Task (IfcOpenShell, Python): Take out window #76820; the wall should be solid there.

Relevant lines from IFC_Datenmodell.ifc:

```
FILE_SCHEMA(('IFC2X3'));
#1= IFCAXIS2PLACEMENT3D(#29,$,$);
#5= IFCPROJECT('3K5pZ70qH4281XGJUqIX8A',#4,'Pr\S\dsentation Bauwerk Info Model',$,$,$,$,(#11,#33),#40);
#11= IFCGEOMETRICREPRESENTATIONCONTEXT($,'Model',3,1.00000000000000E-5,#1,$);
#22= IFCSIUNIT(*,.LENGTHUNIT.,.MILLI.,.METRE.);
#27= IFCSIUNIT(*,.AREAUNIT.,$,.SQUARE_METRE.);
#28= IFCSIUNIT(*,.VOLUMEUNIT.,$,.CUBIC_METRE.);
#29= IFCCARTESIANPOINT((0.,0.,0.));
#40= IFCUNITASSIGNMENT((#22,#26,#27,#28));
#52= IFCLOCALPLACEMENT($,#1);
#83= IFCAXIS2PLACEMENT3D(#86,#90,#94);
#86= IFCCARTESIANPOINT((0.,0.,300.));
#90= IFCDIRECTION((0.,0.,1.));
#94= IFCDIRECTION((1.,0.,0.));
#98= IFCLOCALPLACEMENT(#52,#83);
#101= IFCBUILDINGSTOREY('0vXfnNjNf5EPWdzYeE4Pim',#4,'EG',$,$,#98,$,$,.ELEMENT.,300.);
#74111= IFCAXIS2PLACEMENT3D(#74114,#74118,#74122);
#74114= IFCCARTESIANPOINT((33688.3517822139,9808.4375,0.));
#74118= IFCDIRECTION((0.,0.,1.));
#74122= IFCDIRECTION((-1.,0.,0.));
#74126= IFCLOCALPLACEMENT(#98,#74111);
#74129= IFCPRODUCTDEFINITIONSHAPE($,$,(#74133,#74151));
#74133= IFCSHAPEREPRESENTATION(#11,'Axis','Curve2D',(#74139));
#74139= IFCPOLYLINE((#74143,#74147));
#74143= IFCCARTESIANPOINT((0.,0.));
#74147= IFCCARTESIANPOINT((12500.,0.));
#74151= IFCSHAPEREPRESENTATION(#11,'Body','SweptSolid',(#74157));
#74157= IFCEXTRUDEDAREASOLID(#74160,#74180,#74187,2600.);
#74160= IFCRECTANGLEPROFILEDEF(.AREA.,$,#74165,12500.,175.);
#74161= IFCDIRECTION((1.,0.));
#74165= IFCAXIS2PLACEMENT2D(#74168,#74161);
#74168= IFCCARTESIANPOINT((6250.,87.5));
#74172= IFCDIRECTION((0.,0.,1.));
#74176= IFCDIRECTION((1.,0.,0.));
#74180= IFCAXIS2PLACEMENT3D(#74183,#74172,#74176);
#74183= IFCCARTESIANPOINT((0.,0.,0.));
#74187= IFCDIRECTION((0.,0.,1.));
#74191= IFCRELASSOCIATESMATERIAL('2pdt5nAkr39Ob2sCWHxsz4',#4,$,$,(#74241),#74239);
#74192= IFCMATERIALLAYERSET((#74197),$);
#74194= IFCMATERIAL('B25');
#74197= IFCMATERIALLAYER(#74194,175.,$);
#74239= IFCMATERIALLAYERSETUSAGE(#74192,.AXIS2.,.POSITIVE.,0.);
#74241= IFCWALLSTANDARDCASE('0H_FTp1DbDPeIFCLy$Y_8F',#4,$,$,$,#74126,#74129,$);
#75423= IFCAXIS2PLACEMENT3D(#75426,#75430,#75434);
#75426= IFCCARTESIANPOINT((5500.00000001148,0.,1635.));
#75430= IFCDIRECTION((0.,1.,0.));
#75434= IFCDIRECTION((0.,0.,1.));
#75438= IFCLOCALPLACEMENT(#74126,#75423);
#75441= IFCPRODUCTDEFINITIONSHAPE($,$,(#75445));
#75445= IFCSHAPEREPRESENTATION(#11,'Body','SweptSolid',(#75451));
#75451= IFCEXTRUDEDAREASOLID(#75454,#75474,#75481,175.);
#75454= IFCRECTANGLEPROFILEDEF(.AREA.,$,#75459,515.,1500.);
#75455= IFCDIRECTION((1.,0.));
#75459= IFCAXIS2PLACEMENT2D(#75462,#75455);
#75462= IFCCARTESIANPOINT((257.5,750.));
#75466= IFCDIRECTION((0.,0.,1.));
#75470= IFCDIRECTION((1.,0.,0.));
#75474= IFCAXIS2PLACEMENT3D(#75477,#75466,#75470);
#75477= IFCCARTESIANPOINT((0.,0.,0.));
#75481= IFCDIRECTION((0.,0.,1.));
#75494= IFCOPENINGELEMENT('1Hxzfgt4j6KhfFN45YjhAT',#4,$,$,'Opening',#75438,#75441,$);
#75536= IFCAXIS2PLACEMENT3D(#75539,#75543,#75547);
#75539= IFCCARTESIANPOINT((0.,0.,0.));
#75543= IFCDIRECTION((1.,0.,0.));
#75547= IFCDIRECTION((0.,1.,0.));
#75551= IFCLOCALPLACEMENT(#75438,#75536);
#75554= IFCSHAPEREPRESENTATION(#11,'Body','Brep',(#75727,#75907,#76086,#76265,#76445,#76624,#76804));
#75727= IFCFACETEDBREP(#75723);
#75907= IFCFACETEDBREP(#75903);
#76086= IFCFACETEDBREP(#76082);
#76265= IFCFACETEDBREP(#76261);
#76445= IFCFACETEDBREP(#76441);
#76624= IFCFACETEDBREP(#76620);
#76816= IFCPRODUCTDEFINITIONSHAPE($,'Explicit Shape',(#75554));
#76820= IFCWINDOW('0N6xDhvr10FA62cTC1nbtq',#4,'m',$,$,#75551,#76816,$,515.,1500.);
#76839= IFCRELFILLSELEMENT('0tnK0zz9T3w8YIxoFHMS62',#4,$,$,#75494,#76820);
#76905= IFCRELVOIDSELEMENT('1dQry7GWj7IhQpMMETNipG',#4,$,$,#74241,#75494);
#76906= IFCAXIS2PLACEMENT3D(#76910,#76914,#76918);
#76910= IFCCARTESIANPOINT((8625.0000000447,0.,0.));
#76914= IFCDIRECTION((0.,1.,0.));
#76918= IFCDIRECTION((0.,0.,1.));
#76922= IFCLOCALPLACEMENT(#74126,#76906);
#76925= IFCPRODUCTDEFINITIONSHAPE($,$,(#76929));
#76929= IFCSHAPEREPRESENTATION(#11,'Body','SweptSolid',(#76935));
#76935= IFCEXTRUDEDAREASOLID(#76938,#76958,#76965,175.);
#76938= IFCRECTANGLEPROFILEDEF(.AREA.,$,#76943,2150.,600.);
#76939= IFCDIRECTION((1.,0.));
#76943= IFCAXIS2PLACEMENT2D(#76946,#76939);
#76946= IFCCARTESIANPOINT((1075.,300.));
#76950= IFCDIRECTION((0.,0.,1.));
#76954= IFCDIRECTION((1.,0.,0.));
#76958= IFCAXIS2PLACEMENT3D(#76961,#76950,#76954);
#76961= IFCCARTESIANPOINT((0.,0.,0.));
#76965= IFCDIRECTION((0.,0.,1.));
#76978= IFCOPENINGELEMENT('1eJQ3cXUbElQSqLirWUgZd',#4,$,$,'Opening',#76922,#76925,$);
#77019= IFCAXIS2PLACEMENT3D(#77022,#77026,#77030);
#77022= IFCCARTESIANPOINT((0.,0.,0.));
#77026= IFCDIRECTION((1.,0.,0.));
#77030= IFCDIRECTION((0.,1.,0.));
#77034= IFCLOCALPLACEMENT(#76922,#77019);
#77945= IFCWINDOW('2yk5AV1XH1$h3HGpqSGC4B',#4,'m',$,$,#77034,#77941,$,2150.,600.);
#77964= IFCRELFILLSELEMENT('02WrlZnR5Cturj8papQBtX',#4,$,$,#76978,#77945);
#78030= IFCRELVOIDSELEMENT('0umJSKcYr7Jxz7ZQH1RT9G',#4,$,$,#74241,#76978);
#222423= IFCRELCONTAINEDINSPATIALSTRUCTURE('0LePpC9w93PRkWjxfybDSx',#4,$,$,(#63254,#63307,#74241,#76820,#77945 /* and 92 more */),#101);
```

```python
import ifcopenshell
import ifcopenshell.api.feature
import ifcopenshell.api.root
import ifcopenshell.geom
import ifcopenshell.util.shape

model = ifcopenshell.open("IFC_Datenmodell.ifc")
settings = ifcopenshell.geom.settings()


def volume(element):
    """Net volume in cubic metres, openings subtracted."""
    shape = ifcopenshell.geom.create_shape(settings, element)
    return ifcopenshell.util.shape.get_volume(shape.geometry)


window = model.by_guid("0N6xDhvr10FA62cTC1nbtq")
opening = window.FillsVoids[0].RelatingOpeningElement
wall = opening.VoidsElements[0].RelatingBuildingElement
before = volume(wall)

ifcopenshell.api.root.remove_product(model, product=window)
ifcopenshell.api.feature.remove_feature(model, feature=opening)

after = volume(wall)

print(f"wall volume {before:.3f} -> {after:.3f} m3")

model.write("IFC_Datenmodell_updated.ifc")
```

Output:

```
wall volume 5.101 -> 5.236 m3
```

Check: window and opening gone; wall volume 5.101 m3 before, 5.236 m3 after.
